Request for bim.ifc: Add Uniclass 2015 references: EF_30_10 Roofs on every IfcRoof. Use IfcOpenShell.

First a look at what the model holds.

```python
import ifcopenshell

model = ifcopenshell.open("bim.ifc")
print(model.schema)
print("classifications:", [c.Name for c in model.by_type("IfcClassification")])
for ifc_class in ("IfcDoor", "IfcRoof", "IfcStair", "IfcWall", "IfcWindow"):
    print(ifc_class, len(model.by_type(ifc_class)))
```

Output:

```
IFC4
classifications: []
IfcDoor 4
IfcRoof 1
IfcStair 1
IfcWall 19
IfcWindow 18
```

```python
import ifcopenshell
import ifcopenshell.api.classification

model = ifcopenshell.open("bim.ifc")

system = ifcopenshell.api.classification.add_classification(model, classification="Uniclass 2015")

codes = {
    "IfcRoof": ("EF_30_10", "Roofs"),
}
for ifc_class, (code, name) in codes.items():
    products = model.by_type(ifc_class)
    ifcopenshell.api.classification.add_reference(
        model, products=products, classification=system, identification=code, name=name
    )
    print(code, len(products))

model.write("bim_edited.ifc")
```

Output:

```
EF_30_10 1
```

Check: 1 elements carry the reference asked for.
